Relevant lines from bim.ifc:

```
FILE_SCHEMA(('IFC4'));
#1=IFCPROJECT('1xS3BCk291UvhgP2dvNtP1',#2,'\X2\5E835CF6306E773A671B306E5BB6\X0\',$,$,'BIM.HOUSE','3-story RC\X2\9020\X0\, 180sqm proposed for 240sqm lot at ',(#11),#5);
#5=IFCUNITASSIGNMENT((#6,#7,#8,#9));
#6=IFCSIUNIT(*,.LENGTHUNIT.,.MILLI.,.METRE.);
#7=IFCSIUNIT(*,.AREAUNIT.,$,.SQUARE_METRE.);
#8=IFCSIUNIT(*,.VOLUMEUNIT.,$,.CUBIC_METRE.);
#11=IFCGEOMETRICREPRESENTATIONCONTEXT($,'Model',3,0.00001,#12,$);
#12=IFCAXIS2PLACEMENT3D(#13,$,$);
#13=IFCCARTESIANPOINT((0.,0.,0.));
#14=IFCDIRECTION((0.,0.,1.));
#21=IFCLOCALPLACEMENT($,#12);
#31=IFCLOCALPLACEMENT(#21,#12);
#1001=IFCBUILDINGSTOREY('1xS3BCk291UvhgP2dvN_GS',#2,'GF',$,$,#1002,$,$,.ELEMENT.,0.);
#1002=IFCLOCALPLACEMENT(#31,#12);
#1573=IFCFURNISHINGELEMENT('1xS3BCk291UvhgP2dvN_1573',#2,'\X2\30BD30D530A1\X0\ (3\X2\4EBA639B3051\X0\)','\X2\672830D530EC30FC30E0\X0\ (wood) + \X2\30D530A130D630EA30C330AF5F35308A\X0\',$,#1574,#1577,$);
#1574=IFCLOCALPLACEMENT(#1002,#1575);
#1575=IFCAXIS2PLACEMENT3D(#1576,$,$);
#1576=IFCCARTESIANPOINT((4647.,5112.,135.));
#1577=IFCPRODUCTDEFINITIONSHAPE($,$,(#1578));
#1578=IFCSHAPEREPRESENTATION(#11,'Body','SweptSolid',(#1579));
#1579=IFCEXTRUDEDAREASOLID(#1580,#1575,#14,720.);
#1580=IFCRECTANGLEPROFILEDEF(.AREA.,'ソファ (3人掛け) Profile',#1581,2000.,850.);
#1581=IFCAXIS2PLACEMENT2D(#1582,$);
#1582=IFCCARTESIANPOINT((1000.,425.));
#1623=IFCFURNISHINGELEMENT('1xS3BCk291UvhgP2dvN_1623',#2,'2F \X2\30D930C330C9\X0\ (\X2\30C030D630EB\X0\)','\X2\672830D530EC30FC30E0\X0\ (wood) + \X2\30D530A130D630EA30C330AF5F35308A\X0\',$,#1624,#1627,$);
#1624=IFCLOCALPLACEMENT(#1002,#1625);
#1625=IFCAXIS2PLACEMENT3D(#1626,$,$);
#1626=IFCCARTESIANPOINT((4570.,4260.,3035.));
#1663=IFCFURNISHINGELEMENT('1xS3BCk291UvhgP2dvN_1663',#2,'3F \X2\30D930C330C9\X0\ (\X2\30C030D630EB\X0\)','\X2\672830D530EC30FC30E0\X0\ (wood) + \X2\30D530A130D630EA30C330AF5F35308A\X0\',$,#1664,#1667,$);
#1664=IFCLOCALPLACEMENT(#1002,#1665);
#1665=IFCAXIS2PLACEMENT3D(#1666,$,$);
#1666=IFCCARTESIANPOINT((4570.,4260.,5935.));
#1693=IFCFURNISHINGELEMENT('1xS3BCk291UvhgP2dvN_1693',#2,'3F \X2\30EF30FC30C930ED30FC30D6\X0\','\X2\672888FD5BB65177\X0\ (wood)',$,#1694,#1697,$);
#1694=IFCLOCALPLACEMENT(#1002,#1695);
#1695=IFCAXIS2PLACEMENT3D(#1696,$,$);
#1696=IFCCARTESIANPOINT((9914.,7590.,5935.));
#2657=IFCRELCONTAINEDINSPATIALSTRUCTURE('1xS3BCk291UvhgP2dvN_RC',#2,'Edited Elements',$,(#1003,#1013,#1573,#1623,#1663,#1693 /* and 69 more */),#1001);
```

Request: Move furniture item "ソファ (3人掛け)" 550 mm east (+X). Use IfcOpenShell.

```python
import ifcopenshell
import ifcopenshell.api.geometry
import ifcopenshell.util.placement
import ifcopenshell.util.unit

model = ifcopenshell.open("bim.ifc")
unit_scale = ifcopenshell.util.unit.calculate_unit_scale(model)

item = model.by_guid("1xS3BCk291UvhgP2dvN_1573")
matrix = ifcopenshell.util.placement.get_local_placement(item.ObjectPlacement)
matrix[0, 3] += 0.55 / unit_scale
ifcopenshell.api.geometry.edit_object_placement(model, product=item, matrix=matrix, is_si=False)

print(ifcopenshell.util.placement.get_local_placement(item.ObjectPlacement).round(3) + 0.0)

model.write("bim_rev.ifc")
```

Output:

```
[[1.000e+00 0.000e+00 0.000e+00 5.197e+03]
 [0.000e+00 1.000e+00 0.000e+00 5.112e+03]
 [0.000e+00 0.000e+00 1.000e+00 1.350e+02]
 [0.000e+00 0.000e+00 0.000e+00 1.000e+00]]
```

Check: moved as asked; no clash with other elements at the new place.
